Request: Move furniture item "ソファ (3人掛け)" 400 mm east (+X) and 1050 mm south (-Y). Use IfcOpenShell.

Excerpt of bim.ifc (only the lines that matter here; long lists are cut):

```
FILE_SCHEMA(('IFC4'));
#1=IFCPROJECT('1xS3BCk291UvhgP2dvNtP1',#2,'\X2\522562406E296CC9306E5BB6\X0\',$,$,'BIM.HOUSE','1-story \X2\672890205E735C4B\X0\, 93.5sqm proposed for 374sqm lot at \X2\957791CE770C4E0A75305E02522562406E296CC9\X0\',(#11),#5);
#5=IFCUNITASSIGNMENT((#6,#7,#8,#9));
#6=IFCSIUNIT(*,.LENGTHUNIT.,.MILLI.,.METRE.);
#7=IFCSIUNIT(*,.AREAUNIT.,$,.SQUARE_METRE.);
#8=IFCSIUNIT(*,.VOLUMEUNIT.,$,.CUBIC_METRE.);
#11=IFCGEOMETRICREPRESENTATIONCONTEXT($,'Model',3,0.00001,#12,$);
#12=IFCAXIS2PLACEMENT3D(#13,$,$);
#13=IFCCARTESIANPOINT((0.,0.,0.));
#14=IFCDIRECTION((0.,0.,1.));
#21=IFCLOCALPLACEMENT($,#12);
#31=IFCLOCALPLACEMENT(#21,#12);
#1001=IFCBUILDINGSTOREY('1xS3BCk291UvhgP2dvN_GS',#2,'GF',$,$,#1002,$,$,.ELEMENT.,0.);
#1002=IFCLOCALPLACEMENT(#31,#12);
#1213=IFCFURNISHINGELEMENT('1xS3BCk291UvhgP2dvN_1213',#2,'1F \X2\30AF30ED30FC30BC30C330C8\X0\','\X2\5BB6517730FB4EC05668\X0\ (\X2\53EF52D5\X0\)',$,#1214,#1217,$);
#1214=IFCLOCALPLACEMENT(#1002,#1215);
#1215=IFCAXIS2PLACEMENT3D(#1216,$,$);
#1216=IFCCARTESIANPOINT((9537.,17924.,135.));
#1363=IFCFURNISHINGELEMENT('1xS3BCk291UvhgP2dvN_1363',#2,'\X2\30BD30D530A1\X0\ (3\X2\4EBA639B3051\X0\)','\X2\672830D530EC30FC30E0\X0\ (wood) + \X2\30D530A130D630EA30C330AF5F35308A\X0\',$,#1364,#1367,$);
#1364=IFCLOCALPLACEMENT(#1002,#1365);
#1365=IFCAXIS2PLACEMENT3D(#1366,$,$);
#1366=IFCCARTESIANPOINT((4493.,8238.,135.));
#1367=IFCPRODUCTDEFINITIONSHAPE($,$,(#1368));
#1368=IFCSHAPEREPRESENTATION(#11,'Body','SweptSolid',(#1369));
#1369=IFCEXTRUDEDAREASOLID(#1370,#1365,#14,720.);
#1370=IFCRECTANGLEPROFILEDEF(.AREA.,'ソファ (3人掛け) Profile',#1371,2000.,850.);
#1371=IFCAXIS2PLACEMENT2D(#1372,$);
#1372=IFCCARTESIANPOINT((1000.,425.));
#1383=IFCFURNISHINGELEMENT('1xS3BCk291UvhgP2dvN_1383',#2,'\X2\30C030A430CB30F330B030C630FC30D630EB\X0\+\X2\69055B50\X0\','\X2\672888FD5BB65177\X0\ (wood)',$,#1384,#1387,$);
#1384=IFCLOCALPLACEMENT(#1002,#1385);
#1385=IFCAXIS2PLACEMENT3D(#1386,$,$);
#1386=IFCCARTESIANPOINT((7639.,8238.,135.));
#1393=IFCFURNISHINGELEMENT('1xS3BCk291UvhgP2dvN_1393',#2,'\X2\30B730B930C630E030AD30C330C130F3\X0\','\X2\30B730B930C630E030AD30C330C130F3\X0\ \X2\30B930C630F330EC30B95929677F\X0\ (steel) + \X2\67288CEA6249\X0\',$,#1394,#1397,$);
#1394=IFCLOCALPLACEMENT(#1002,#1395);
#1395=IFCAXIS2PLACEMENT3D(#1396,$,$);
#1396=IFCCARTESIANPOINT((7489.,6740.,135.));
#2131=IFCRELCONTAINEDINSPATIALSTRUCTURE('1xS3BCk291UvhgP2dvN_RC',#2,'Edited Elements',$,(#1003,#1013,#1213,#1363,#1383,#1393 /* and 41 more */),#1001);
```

```python
import ifcopenshell
import ifcopenshell.api.geometry
import ifcopenshell.util.placement
import ifcopenshell.util.unit

model = ifcopenshell.open("bim.ifc")
unit_scale = ifcopenshell.util.unit.calculate_unit_scale(model)

item = model.by_guid("1xS3BCk291UvhgP2dvN_1363")
matrix = ifcopenshell.util.placement.get_local_placement(item.ObjectPlacement)
matrix[0, 3] += 0.4 / unit_scale
matrix[1, 3] -= 1.05 / unit_scale
ifcopenshell.api.geometry.edit_object_placement(model, product=item, matrix=matrix, is_si=False)

print(ifcopenshell.util.placement.get_local_placement(item.ObjectPlacement).round(3) + 0.0)

model.write("bim_updated.ifc")
```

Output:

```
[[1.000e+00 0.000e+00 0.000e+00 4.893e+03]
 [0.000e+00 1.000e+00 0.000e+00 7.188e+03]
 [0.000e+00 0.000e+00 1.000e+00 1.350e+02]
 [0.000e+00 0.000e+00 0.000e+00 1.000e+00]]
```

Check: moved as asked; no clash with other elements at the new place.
